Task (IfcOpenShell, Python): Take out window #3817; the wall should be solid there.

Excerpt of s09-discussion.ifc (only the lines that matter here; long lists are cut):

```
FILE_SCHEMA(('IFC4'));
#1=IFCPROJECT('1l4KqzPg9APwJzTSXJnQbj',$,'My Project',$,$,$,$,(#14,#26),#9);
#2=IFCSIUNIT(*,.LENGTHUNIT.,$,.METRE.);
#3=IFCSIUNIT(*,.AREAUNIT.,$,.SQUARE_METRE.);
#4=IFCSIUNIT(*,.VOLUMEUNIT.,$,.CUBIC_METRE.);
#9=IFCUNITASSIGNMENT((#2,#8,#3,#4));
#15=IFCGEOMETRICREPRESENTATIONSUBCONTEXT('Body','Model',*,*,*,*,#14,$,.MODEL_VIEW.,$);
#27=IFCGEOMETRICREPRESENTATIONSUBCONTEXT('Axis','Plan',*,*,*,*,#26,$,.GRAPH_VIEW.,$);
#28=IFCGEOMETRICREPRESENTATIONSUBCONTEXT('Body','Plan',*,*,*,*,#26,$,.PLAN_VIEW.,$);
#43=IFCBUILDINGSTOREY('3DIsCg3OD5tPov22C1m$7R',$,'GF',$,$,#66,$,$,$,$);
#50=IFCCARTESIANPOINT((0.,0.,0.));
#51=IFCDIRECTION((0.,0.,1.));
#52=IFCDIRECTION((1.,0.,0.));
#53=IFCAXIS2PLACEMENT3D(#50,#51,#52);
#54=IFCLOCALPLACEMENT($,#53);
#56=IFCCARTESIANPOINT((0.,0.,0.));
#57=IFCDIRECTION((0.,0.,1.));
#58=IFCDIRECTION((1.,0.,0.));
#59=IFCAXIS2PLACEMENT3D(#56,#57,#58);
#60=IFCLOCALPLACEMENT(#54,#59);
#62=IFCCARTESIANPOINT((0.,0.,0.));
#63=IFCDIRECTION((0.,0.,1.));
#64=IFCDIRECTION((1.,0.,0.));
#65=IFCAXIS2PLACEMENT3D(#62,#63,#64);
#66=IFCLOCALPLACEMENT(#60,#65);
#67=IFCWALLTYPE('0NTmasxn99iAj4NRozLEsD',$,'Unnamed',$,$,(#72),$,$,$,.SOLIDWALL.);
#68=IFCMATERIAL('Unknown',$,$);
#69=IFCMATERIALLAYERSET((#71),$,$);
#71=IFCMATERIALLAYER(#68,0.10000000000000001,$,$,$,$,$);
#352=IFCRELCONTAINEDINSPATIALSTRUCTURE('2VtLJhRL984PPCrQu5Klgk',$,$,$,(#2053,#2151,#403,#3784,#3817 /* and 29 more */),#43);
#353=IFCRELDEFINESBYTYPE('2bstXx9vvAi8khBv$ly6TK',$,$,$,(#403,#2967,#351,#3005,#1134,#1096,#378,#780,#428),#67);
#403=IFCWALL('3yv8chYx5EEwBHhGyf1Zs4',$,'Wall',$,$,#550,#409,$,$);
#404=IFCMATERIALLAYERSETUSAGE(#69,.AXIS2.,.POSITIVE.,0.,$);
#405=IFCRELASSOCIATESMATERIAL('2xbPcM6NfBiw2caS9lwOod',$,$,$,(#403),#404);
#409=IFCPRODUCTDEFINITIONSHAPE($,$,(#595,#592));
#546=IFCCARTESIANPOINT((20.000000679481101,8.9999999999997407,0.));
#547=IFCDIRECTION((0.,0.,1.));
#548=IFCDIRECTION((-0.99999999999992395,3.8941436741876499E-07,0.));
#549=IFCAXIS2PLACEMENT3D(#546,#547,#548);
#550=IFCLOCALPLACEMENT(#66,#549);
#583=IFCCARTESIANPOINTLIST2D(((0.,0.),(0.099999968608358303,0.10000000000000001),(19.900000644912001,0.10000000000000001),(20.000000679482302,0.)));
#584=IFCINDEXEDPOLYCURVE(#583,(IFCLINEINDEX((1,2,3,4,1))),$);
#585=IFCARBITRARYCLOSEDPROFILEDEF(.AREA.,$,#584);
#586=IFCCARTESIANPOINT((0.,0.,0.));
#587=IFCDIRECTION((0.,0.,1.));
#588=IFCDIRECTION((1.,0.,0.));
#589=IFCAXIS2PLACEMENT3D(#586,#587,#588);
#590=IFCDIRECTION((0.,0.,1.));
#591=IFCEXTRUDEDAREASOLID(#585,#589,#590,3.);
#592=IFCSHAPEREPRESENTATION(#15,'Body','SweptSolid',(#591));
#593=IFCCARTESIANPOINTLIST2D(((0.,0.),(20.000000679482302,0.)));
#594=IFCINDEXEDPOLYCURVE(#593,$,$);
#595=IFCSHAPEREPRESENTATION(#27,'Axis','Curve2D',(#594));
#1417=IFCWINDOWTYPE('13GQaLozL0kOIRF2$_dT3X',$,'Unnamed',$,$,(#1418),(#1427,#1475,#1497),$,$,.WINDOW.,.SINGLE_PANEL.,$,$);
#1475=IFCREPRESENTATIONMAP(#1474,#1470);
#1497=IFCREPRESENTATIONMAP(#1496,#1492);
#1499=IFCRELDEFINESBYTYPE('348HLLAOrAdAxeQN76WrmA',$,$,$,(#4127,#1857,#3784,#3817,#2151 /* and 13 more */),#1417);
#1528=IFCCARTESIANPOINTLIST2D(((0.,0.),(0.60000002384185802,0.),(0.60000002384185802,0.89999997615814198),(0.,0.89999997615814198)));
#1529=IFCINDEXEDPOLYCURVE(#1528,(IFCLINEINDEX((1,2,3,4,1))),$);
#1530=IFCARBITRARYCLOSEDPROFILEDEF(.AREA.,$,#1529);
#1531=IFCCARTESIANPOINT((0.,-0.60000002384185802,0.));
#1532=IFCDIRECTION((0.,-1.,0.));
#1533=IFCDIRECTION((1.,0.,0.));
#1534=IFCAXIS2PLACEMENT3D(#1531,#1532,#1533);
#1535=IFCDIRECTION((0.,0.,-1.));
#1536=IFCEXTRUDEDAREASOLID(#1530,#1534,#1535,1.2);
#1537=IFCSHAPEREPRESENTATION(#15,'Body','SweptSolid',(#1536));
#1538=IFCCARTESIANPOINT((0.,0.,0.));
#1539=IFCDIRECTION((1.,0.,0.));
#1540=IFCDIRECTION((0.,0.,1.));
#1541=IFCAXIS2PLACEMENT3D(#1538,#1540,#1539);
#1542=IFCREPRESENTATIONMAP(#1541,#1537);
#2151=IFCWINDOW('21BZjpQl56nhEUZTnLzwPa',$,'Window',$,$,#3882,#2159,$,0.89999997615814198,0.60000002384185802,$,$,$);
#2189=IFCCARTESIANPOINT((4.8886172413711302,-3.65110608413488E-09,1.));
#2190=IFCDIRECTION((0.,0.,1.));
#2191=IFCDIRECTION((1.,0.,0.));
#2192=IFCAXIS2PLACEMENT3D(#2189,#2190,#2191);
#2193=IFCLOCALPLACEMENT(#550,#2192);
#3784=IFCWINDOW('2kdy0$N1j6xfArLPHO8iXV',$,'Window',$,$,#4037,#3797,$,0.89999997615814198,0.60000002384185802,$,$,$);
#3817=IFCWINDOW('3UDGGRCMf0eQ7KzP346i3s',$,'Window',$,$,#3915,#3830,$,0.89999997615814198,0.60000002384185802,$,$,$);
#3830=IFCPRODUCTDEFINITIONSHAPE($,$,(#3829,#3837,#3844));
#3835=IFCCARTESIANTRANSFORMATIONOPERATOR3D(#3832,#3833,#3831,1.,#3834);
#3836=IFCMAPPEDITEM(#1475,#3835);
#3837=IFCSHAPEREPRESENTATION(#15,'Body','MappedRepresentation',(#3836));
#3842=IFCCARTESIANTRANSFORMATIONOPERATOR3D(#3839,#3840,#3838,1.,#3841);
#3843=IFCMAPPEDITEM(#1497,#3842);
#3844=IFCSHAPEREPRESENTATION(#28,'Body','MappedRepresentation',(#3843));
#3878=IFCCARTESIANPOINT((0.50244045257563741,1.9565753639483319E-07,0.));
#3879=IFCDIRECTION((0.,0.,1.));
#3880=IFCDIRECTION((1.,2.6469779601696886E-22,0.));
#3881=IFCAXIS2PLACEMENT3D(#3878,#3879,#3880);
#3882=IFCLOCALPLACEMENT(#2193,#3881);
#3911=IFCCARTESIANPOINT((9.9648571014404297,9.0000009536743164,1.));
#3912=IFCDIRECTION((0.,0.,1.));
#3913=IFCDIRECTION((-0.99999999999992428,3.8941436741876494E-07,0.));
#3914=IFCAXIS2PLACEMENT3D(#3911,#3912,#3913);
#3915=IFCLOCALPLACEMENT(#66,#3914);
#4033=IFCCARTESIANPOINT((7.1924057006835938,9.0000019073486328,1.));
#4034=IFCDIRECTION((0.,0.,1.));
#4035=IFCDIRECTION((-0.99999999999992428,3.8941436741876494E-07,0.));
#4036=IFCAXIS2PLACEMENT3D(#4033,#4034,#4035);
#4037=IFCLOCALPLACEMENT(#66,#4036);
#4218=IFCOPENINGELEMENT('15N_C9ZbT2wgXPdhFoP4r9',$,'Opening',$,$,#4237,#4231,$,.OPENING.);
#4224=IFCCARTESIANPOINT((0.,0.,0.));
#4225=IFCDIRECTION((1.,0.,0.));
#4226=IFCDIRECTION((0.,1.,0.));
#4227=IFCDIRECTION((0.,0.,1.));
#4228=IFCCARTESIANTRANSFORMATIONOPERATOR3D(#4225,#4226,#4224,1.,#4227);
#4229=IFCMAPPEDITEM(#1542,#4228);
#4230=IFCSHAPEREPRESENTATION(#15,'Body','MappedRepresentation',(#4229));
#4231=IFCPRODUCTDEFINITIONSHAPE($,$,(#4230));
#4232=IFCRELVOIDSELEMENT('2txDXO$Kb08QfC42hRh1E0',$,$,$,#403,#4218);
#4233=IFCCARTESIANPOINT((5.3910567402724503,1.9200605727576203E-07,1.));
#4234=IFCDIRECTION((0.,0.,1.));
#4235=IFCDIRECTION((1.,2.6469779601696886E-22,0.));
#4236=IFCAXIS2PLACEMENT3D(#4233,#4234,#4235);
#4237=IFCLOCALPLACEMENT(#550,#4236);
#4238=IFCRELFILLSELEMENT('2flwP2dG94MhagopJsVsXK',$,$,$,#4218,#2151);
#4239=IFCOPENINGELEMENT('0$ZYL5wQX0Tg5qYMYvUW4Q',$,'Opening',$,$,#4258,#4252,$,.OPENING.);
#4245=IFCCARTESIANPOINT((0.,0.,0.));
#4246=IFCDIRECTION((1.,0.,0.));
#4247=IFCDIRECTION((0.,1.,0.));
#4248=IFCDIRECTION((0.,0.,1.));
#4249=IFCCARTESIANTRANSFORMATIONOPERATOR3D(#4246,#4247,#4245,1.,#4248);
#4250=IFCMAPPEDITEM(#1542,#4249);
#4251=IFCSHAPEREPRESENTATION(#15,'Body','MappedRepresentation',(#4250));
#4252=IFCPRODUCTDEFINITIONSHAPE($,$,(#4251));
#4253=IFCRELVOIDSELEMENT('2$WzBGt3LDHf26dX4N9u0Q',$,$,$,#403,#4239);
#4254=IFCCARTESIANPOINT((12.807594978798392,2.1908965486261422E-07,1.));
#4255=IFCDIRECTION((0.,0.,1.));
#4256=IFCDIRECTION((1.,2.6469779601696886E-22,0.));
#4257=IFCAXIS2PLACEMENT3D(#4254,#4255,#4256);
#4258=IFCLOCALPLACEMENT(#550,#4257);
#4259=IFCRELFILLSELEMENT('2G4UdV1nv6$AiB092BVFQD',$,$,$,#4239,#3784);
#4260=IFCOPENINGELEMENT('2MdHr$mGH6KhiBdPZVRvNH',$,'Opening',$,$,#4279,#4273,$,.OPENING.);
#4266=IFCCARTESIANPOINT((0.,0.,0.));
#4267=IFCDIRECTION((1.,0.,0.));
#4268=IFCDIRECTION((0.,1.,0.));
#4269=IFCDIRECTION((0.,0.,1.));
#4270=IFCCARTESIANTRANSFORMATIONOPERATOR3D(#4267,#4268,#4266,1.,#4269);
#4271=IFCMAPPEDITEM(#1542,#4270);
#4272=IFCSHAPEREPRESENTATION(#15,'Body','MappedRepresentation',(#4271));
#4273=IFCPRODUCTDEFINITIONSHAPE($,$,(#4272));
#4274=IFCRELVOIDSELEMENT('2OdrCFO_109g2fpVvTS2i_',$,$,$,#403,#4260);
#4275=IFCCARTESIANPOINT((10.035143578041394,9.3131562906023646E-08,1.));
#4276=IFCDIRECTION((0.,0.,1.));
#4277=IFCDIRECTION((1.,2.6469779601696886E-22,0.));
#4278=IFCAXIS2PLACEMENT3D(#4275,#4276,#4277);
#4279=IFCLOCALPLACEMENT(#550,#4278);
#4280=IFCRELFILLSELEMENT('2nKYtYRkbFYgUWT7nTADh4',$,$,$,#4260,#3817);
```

```python
import ifcopenshell
import ifcopenshell.api.feature
import ifcopenshell.api.root
import ifcopenshell.geom
import ifcopenshell.util.shape

model = ifcopenshell.open("s09-discussion.ifc")
settings = ifcopenshell.geom.settings()


def volume(element):
    """Net volume in cubic metres, openings subtracted."""
    shape = ifcopenshell.geom.create_shape(settings, element)
    return ifcopenshell.util.shape.get_volume(shape.geometry)


window = model.by_guid("3UDGGRCMf0eQ7KzP346i3s")
opening = window.FillsVoids[0].RelatingOpeningElement
wall = opening.VoidsElements[0].RelatingBuildingElement
before = volume(wall)

ifcopenshell.api.root.remove_product(model, product=window)
ifcopenshell.api.feature.remove_feature(model, feature=opening)

after = volume(wall)

print(f"wall volume {before:.3f} -> {after:.3f} m3")

model.write("s09-discussion-out.ifc")
```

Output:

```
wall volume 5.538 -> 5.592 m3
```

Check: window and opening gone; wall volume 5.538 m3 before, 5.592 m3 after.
